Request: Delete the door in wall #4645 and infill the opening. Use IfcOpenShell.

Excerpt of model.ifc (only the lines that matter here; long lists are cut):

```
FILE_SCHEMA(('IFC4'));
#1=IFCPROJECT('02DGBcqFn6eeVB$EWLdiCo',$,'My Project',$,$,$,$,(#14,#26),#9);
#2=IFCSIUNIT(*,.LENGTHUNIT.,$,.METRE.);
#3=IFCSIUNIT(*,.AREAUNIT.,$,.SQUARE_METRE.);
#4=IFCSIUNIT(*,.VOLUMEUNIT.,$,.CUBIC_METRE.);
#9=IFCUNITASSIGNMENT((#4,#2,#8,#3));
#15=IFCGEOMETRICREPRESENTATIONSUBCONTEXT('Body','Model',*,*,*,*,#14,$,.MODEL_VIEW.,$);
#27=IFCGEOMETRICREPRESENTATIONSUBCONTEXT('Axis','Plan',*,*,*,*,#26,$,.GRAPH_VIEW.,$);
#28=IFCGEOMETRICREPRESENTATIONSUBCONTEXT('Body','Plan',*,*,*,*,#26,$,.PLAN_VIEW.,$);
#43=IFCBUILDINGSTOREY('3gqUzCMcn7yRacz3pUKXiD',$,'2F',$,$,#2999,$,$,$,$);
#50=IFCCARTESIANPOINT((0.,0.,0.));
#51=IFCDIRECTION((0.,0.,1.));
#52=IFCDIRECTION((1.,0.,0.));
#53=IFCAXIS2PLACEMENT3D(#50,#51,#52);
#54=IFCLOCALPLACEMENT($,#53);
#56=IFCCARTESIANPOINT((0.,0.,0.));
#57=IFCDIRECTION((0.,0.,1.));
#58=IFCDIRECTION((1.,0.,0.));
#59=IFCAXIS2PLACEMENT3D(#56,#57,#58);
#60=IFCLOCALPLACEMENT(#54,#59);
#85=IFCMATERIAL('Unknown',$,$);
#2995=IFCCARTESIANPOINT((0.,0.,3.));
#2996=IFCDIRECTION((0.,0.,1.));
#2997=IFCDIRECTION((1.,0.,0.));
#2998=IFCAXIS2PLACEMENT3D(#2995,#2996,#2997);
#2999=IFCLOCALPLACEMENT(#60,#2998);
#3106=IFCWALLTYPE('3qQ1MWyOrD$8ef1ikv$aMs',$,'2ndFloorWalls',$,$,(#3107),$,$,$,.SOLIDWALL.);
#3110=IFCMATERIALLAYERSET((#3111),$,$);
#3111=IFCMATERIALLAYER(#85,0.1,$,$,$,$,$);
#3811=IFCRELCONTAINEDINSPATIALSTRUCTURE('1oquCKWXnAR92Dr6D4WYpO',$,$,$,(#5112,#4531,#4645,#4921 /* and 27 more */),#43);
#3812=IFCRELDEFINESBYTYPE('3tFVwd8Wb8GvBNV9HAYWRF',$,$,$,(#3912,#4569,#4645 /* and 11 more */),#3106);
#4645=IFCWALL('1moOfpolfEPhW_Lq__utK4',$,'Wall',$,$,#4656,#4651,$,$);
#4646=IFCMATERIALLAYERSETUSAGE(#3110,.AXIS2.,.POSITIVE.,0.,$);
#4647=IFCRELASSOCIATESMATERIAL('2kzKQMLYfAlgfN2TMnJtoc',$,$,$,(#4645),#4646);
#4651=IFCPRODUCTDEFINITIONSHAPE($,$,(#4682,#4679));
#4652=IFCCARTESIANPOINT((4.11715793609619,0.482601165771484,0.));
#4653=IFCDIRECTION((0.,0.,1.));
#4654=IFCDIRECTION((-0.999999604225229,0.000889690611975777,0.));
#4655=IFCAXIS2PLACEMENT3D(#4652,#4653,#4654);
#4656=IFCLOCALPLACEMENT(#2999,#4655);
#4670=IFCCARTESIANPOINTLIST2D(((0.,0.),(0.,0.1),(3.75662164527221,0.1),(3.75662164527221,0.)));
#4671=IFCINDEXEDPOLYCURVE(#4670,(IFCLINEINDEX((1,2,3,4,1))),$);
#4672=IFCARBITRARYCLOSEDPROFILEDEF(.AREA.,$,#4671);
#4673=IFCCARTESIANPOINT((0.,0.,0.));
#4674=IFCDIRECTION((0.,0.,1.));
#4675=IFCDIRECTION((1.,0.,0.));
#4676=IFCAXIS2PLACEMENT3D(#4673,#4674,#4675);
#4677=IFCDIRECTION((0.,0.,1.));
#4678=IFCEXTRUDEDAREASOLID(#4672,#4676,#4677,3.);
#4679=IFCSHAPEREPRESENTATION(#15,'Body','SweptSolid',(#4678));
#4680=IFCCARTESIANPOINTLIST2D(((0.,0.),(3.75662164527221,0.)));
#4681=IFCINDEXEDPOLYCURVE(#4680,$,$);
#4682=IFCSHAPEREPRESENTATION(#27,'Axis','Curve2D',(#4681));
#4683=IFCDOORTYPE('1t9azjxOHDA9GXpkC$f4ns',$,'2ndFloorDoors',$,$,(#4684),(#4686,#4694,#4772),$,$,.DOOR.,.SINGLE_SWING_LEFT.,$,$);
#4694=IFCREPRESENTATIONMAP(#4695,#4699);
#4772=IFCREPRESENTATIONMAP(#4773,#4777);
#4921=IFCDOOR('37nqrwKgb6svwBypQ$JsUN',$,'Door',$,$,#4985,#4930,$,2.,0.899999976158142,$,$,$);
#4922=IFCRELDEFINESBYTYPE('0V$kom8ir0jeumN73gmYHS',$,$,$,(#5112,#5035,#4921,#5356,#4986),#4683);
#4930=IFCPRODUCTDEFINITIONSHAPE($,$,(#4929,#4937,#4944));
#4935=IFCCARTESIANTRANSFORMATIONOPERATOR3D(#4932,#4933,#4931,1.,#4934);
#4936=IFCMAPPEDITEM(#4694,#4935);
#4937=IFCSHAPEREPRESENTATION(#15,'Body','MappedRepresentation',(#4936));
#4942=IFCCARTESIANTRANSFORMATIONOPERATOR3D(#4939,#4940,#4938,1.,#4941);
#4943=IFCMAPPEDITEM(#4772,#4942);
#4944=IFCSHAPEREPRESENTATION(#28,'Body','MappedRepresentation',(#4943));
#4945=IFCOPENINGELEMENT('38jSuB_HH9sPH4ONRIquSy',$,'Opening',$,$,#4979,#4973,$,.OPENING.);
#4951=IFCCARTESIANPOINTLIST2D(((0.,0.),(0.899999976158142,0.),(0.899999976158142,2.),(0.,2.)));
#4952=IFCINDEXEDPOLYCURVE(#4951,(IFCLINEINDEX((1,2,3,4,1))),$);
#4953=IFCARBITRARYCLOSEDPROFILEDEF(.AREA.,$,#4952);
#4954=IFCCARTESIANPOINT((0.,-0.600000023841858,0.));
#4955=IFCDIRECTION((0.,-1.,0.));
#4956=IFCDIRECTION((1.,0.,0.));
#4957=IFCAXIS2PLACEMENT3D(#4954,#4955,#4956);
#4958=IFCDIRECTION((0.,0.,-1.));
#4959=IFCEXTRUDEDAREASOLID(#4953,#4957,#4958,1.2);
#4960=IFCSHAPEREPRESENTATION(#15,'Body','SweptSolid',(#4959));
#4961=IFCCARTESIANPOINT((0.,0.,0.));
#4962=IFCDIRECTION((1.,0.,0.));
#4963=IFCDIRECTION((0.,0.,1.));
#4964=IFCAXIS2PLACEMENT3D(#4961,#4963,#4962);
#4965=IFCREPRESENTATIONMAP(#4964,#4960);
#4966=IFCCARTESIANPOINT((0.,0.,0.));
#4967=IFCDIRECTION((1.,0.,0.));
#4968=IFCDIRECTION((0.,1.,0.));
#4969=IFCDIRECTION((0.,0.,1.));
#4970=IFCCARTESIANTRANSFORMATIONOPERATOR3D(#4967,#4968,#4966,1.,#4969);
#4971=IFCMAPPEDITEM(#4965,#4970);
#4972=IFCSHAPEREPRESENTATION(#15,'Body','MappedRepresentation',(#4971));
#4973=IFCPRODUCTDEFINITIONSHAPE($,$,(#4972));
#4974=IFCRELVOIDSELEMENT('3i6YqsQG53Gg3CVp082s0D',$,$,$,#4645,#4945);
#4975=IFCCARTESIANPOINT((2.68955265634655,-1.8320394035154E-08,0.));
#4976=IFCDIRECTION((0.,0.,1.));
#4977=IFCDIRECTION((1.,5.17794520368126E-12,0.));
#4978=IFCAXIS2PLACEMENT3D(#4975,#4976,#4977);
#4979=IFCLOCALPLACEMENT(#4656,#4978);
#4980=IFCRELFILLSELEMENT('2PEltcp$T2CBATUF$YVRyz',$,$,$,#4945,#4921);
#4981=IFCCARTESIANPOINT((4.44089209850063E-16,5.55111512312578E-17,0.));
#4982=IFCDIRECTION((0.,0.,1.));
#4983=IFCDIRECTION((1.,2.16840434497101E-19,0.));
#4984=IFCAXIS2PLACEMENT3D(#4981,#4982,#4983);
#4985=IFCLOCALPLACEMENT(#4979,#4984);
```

```python
import ifcopenshell
import ifcopenshell.api.feature
import ifcopenshell.api.root
import ifcopenshell.geom
import ifcopenshell.util.shape

model = ifcopenshell.open("model.ifc")
settings = ifcopenshell.geom.settings()


def volume(element):
    """Net volume in cubic metres, openings subtracted."""
    shape = ifcopenshell.geom.create_shape(settings, element)
    return ifcopenshell.util.shape.get_volume(shape.geometry)


door = model.by_guid("37nqrwKgb6svwBypQ$JsUN")
opening = door.FillsVoids[0].RelatingOpeningElement
wall = opening.VoidsElements[0].RelatingBuildingElement
before = volume(wall)

ifcopenshell.api.root.remove_product(model, product=door)
ifcopenshell.api.feature.remove_feature(model, feature=opening)

after = volume(wall)

print(f"wall volume {before:.3f} -> {after:.3f} m3")

model.write("model-out.ifc")
```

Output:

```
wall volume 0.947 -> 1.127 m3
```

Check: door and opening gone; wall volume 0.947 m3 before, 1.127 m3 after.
